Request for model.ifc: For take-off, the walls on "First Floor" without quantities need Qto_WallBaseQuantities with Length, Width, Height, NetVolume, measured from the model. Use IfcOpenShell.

First a look at what the model holds.

```python
import ifcopenshell
import ifcopenshell.util.element
import ifcopenshell.util.unit

model = ifcopenshell.open("model.ifc")
print(model.schema)
for unit_type in ("LENGTHUNIT", "AREAUNIT", "VOLUMEUNIT"):
    print(unit_type, ifcopenshell.util.unit.calculate_unit_scale(model, unit_type))
storey = next(s for s in model.by_type("IfcBuildingStorey") if s.Name == "First Floor")
walls = [e for e in ifcopenshell.util.element.get_decomposition(storey) if e.is_a("IfcWall")]
for e in sorted(walls, key=lambda e: e.id()):
    print(e.id(), e.is_a(), e.Name, list(ifcopenshell.util.element.get_psets(e, qtos_only=True)), sep=" | ")
```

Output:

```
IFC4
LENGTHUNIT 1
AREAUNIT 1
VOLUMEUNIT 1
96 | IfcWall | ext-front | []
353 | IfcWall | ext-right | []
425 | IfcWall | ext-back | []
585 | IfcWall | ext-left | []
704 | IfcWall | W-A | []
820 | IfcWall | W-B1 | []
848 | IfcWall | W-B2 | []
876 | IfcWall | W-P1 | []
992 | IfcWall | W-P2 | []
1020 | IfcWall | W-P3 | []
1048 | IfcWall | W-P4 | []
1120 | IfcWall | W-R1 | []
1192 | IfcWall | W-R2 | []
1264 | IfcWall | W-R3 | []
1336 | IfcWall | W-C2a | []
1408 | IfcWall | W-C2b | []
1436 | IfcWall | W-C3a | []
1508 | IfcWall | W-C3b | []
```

```python
import ifcopenshell
import ifcopenshell.api.pset
import ifcopenshell.geom
import ifcopenshell.util.element
import ifcopenshell.util.shape
import ifcopenshell.util.unit

model = ifcopenshell.open("model.ifc")
unit_scale = ifcopenshell.util.unit.calculate_unit_scale(model)
volume_scale = ifcopenshell.util.unit.calculate_unit_scale(model, "VOLUMEUNIT")
settings = ifcopenshell.geom.settings()

storey = next(s for s in model.by_type("IfcBuildingStorey") if s.Name == "First Floor")
walls = [e for e in ifcopenshell.util.element.get_decomposition(storey) if e.is_a("IfcWall")]

for e in sorted(walls, key=lambda e: e.id()):
    if ifcopenshell.util.element.get_psets(e, qtos_only=True, should_inherit=False):
        continue
    # Geometry comes back in metres, in the element's own axes.
    shape = ifcopenshell.geom.create_shape(settings, e)
    values = {
        "Length": ifcopenshell.util.shape.get_x(shape.geometry) / unit_scale,
        "Width": ifcopenshell.util.shape.get_y(shape.geometry) / unit_scale,
        "Height": ifcopenshell.util.shape.get_z(shape.geometry) / unit_scale,
        "NetVolume": ifcopenshell.util.shape.get_volume(shape.geometry) / volume_scale,
    }
    qto = ifcopenshell.api.pset.add_qto(model, product=e, name="Qto_WallBaseQuantities")
    ifcopenshell.api.pset.edit_qto(model, qto=qto, properties=values)
    print(e.id(), {k: round(v, 3) for k, v in values.items()})

model.write("model_edited.ifc")
```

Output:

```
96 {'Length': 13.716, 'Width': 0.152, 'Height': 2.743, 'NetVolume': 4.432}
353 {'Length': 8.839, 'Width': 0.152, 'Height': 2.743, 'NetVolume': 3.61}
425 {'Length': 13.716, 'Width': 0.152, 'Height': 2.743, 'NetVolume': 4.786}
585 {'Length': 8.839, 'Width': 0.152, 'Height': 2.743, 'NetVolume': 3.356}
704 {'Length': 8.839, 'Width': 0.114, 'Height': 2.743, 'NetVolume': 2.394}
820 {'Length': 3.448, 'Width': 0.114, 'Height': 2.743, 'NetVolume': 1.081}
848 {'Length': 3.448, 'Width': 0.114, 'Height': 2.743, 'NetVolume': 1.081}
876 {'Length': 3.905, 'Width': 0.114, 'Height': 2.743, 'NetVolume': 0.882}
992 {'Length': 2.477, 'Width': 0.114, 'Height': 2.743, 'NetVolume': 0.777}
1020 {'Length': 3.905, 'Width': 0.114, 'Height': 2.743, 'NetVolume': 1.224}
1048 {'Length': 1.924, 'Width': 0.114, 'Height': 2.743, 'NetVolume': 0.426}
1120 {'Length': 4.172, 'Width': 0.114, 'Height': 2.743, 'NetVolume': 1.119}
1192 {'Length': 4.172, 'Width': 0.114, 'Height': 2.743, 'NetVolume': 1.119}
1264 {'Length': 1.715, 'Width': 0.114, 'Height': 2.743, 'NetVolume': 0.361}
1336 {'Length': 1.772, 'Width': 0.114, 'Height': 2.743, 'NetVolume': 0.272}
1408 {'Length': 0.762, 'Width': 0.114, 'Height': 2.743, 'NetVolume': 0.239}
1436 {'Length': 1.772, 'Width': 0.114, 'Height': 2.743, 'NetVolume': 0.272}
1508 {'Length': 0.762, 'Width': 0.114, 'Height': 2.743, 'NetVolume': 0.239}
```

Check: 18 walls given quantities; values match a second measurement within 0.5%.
